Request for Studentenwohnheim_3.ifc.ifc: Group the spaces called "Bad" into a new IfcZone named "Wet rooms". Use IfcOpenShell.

First a look at what the model holds.

```python
import ifcopenshell

model = ifcopenshell.open("Studentenwohnheim_3.ifc.ifc")
print(model.schema)
seen = {}
for space in model.by_type("IfcSpace"):
    seen[space.LongName] = seen.get(space.LongName, 0) + 1
for name, count in sorted(seen.items(), key=str):
    print(count, "x", name)
print("zones:", [z.Name for z in model.by_type("IfcZone")][:20])
```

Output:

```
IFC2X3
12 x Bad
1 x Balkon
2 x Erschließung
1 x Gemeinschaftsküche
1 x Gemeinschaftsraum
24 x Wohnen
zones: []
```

```python
import ifcopenshell
import ifcopenshell.api.group
import ifcopenshell.api.root

model = ifcopenshell.open("Studentenwohnheim_3.ifc.ifc")

names = {"Bad"}
spaces = [s for s in model.by_type("IfcSpace") if s.LongName in names]

zone = ifcopenshell.api.root.create_entity(model, ifc_class="IfcZone", name="Wet rooms")
ifcopenshell.api.group.assign_group(model, products=spaces, group=zone)
print(len(spaces), "spaces in", zone.Name)

model.write("Studentenwohnheim_3.ifc_v2.ifc")
```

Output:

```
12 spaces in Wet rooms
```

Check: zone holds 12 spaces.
